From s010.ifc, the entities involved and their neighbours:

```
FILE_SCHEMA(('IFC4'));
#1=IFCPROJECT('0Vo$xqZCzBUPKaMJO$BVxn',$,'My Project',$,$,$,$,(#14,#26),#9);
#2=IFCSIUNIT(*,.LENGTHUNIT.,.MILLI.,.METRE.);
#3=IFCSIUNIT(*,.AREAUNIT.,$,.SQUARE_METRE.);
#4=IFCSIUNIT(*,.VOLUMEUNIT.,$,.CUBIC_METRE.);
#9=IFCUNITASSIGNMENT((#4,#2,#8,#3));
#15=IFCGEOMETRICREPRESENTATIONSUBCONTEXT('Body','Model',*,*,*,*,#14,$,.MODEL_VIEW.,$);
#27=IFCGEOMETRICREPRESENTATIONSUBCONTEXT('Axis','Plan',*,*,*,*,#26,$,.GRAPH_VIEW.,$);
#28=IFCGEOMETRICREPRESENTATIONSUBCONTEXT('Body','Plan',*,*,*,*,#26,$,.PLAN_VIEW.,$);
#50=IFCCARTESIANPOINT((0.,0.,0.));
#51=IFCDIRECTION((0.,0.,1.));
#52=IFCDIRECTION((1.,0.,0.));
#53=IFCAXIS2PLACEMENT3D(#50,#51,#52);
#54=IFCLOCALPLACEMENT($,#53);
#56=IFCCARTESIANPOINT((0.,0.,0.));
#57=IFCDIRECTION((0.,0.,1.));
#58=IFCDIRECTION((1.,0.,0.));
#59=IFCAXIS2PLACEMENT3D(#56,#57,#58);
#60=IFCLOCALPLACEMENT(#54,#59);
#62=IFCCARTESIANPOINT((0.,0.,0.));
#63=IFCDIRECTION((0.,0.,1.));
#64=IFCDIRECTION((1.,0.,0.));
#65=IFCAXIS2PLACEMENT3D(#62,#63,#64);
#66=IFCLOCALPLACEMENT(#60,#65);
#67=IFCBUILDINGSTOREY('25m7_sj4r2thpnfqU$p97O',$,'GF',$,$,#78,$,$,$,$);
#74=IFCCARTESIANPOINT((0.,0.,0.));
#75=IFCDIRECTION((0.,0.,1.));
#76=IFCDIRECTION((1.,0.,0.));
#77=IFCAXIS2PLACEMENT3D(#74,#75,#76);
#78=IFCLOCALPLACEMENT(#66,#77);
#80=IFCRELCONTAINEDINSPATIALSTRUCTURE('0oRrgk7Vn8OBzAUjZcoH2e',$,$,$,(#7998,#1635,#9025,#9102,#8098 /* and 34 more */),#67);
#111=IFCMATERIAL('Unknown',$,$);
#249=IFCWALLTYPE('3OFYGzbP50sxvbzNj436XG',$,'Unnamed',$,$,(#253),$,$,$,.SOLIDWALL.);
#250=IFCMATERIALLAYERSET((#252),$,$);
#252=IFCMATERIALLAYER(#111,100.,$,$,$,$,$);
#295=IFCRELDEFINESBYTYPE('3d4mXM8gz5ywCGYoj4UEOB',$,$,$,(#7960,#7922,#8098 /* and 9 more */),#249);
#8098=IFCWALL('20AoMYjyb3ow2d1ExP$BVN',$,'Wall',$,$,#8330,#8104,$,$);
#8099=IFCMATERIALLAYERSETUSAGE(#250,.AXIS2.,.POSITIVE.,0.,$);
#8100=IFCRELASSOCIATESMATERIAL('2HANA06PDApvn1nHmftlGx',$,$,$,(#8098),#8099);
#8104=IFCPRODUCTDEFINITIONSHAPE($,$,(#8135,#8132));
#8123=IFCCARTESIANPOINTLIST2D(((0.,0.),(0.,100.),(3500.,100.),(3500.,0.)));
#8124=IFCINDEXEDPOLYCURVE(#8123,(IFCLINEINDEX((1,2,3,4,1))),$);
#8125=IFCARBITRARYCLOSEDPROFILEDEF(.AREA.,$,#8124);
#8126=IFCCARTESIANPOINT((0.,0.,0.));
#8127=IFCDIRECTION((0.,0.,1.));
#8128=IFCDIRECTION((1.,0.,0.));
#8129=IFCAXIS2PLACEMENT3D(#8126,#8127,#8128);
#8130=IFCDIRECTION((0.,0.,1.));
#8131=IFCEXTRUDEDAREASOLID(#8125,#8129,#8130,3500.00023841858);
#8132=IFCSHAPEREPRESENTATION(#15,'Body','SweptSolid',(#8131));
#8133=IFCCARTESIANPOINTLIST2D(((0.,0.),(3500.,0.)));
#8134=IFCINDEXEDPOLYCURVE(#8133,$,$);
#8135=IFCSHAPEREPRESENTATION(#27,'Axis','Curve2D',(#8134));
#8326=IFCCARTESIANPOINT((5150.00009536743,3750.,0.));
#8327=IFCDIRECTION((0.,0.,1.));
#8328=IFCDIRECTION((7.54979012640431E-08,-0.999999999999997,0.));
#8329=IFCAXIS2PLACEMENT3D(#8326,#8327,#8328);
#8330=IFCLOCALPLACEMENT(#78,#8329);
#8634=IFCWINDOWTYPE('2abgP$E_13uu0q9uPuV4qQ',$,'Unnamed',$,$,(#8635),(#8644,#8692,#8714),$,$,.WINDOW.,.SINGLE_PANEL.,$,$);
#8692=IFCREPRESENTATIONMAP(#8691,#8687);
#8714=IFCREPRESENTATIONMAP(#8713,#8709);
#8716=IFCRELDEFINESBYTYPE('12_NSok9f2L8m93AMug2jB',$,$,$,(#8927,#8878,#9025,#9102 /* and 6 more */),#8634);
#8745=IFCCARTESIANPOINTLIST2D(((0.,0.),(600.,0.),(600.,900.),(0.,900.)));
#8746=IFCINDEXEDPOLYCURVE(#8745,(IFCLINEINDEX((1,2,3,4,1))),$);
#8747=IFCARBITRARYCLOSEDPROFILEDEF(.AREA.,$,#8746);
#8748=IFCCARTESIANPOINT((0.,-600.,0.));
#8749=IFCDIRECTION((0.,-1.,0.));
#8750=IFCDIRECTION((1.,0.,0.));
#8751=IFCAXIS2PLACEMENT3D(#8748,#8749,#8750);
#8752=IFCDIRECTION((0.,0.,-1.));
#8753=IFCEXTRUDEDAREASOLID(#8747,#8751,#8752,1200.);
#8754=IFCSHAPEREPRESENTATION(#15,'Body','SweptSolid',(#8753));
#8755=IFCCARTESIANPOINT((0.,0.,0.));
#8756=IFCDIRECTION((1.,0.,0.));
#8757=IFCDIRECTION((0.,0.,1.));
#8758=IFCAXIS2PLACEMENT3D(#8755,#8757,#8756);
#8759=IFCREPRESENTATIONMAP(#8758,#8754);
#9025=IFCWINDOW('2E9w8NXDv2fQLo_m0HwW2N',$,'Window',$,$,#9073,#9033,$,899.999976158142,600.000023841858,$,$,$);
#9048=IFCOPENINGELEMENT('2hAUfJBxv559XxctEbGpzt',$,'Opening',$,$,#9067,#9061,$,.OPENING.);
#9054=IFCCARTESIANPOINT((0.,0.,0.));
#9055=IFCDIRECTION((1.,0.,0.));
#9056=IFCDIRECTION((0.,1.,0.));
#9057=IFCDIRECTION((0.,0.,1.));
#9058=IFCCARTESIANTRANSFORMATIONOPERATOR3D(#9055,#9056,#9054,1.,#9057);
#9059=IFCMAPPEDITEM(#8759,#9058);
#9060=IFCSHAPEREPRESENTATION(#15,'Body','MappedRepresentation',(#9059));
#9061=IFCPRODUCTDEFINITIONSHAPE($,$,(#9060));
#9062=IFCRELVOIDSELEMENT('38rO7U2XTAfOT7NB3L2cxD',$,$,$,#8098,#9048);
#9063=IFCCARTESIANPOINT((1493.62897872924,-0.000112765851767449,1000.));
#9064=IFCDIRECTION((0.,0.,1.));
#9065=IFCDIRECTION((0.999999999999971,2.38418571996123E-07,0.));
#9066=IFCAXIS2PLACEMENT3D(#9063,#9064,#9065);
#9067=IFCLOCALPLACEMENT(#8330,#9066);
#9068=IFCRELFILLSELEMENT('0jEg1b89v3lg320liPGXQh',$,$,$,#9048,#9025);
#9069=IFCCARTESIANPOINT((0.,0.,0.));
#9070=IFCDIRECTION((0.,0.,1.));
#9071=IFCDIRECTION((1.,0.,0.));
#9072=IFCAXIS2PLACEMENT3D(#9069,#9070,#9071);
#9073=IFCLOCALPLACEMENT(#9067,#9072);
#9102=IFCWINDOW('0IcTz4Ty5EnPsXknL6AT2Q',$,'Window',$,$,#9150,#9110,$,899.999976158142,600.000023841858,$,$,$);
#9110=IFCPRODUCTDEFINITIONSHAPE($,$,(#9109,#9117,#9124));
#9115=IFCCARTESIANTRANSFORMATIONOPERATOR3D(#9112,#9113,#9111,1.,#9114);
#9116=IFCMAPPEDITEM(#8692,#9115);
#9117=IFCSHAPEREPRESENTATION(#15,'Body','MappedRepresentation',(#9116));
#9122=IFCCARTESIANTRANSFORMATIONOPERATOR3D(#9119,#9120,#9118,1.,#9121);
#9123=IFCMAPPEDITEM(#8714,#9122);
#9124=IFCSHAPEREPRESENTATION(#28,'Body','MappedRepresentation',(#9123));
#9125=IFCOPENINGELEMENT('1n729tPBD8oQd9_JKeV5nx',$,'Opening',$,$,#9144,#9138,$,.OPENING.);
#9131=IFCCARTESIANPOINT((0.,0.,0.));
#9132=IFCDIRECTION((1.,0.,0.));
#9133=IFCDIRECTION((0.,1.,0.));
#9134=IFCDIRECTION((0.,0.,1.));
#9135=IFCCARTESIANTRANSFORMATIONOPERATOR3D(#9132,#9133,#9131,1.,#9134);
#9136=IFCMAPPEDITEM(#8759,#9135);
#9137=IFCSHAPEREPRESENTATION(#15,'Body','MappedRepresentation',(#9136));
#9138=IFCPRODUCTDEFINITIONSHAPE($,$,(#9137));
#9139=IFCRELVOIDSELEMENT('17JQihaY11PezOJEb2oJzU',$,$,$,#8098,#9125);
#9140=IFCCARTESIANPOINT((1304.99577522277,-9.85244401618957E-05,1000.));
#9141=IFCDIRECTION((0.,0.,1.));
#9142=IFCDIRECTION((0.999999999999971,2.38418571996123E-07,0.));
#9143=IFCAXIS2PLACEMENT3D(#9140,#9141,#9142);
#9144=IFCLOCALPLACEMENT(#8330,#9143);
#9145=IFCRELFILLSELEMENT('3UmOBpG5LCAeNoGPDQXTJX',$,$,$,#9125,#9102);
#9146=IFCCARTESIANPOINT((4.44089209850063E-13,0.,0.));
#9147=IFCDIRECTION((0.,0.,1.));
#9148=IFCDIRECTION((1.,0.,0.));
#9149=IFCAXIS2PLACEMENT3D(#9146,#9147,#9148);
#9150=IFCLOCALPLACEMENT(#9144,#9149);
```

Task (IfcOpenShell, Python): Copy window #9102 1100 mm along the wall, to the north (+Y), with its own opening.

```python
import ifcopenshell
import ifcopenshell.api.feature
import ifcopenshell.api.geometry
import ifcopenshell.api.root
import ifcopenshell.geom
import ifcopenshell.util.element
import ifcopenshell.util.placement
import ifcopenshell.util.shape

model = ifcopenshell.open("s010.ifc")
settings = ifcopenshell.geom.settings()


def volume(element):
    """Net volume in cubic metres, openings subtracted."""
    shape = ifcopenshell.geom.create_shape(settings, element)
    return ifcopenshell.util.shape.get_volume(shape.geometry)


window = model.by_guid("0IcTz4Ty5EnPsXknL6AT2Q")
opening = window.FillsVoids[0].RelatingOpeningElement
wall = opening.VoidsElements[0].RelatingBuildingElement
before = volume(wall)
shift = ifcopenshell.util.placement.get_local_placement(wall.ObjectPlacement)[:3, 0] * -1100.0

# copy_class copies the void relationship, type, container and properties, but no geometry.
new_opening = ifcopenshell.api.root.copy_class(model, product=opening)
new_opening.Representation = ifcopenshell.util.element.copy_deep(
    model, opening.Representation, exclude=["IfcGeometricRepresentationContext", "IfcRepresentationMap"]
)
new_window = ifcopenshell.api.root.copy_class(model, product=window)
new_window.Representation = ifcopenshell.util.element.copy_deep(
    model, window.Representation, exclude=["IfcGeometricRepresentationContext", "IfcRepresentationMap"]
)
ifcopenshell.api.feature.add_filling(model, opening=new_opening, element=new_window)

for old, new in ((opening, new_opening), (window, new_window)):
    matrix = ifcopenshell.util.placement.get_local_placement(old.ObjectPlacement)
    matrix[:3, 3] += shift
    ifcopenshell.api.geometry.edit_object_placement(model, product=new, matrix=matrix, is_si=False)

after = volume(wall)

print(f"wall volume {before:.3f} -> {after:.3f} m3")

model.write("s010_v2.ifc")
```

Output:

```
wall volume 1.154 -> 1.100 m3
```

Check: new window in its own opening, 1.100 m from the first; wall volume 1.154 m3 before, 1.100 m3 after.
